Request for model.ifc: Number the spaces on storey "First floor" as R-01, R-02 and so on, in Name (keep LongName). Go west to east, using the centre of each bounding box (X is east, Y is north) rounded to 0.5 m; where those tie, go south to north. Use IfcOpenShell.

First a look at what the model holds.

```python
import ifcopenshell
import ifcopenshell.util.element
import ifcopenshell.util.placement

model = ifcopenshell.open("model.ifc")
print(model.schema)
storey = next(s for s in model.by_type("IfcBuildingStorey") if s.Name == "First floor")
spaces = [e for e in ifcopenshell.util.element.get_decomposition(storey) if e.is_a("IfcSpace")]
for e in sorted(spaces, key=lambda e: e.id()):
    origin = ifcopenshell.util.placement.get_local_placement(e.ObjectPlacement)[:3, 3]
    print(e.id(), e.Name, e.LongName, origin.round(2) + 0.0, sep=" | ")
```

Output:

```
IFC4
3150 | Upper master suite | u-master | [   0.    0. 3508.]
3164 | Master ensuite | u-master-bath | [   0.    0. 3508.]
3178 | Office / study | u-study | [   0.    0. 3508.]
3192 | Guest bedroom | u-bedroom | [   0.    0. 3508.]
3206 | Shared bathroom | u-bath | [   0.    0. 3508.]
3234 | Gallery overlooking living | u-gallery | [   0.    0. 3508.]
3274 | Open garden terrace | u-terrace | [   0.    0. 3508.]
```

```python
import ifcopenshell
import ifcopenshell.geom
import ifcopenshell.util.element
import ifcopenshell.util.shape

model = ifcopenshell.open("model.ifc")
settings = ifcopenshell.geom.settings()
settings.set("use-world-coords", True)


def centre(element):
    shape = ifcopenshell.geom.create_shape(settings, element)
    return ifcopenshell.util.shape.get_bbox_centroid(shape.geometry)


storey = next(s for s in model.by_type("IfcBuildingStorey") if s.Name == "First floor")
spaces = [e for e in ifcopenshell.util.element.get_decomposition(storey) if e.is_a("IfcSpace")]

# Insertion points can sit at a corner or the storey origin, so sort by the geometry (in metres).
centres = {e: centre(e) for e in spaces}
spaces.sort(key=lambda e: (round(centres[e][0] / 0.5), centres[e][1]))

for i, e in enumerate(spaces, start=1):
    number = f"R-{i:02d}"
    e.Name = number
    print(e.id(), number)

model.write("model_v2.ifc")
```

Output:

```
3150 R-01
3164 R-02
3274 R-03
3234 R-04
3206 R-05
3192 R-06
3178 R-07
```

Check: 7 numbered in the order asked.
